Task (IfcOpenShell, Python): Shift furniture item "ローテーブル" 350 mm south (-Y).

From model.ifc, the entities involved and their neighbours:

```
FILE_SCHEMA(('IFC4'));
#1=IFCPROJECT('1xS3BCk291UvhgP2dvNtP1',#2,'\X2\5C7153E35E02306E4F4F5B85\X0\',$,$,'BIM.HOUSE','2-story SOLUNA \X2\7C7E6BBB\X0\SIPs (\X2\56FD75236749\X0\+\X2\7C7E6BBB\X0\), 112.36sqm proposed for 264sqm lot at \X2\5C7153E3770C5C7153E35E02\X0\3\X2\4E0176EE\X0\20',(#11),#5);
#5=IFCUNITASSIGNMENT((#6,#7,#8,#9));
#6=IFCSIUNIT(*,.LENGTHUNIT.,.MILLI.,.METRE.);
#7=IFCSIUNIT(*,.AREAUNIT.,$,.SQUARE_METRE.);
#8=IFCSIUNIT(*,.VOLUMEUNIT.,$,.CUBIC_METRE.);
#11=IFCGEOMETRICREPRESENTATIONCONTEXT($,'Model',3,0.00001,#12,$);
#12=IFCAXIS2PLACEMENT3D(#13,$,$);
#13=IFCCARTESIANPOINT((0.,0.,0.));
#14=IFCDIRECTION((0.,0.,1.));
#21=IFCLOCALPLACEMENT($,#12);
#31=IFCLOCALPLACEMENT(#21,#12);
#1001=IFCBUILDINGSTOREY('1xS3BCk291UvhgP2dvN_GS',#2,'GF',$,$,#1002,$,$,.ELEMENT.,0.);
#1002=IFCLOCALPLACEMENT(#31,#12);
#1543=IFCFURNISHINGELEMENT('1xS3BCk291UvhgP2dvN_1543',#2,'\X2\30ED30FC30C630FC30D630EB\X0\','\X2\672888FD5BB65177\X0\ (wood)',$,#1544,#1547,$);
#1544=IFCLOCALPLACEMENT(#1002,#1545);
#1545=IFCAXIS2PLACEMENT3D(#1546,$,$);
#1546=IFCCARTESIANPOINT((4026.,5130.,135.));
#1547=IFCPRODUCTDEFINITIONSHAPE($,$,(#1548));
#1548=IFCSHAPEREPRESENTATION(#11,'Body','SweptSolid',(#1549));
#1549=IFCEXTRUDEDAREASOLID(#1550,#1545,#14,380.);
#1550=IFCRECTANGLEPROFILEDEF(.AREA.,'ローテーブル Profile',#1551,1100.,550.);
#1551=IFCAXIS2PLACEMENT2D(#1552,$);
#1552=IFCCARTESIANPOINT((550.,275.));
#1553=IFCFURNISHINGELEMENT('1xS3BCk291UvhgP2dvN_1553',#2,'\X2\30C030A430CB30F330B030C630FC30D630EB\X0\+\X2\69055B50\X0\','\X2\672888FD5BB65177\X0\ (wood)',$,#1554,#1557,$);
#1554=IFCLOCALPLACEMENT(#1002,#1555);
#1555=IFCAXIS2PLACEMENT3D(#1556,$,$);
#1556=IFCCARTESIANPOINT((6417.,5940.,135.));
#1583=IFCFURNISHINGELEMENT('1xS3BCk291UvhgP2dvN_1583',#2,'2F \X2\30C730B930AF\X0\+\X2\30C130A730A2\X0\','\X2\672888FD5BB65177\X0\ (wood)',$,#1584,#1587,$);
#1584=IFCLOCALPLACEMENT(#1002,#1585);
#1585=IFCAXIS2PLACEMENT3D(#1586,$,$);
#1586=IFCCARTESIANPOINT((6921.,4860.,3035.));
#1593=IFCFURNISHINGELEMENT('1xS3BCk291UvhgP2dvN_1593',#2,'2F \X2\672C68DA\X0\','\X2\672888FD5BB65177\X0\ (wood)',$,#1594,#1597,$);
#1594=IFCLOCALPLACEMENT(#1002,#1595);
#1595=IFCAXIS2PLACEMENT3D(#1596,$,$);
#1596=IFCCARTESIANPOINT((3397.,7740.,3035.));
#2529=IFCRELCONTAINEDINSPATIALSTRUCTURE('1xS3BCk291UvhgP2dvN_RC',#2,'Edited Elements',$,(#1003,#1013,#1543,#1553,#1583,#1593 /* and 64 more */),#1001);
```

```python
import ifcopenshell
import ifcopenshell.api.geometry
import ifcopenshell.util.placement
import ifcopenshell.util.unit

model = ifcopenshell.open("model.ifc")
unit_scale = ifcopenshell.util.unit.calculate_unit_scale(model)

item = model.by_guid("1xS3BCk291UvhgP2dvN_1543")
matrix = ifcopenshell.util.placement.get_local_placement(item.ObjectPlacement)
matrix[1, 3] -= 0.35 / unit_scale
ifcopenshell.api.geometry.edit_object_placement(model, product=item, matrix=matrix, is_si=False)

print(ifcopenshell.util.placement.get_local_placement(item.ObjectPlacement).round(3) + 0.0)

model.write("model_edited.ifc")
```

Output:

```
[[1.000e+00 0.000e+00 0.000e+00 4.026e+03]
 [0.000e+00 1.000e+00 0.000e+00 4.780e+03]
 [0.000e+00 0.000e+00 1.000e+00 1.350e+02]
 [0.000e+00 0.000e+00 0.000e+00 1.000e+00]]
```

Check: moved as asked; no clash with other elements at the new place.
